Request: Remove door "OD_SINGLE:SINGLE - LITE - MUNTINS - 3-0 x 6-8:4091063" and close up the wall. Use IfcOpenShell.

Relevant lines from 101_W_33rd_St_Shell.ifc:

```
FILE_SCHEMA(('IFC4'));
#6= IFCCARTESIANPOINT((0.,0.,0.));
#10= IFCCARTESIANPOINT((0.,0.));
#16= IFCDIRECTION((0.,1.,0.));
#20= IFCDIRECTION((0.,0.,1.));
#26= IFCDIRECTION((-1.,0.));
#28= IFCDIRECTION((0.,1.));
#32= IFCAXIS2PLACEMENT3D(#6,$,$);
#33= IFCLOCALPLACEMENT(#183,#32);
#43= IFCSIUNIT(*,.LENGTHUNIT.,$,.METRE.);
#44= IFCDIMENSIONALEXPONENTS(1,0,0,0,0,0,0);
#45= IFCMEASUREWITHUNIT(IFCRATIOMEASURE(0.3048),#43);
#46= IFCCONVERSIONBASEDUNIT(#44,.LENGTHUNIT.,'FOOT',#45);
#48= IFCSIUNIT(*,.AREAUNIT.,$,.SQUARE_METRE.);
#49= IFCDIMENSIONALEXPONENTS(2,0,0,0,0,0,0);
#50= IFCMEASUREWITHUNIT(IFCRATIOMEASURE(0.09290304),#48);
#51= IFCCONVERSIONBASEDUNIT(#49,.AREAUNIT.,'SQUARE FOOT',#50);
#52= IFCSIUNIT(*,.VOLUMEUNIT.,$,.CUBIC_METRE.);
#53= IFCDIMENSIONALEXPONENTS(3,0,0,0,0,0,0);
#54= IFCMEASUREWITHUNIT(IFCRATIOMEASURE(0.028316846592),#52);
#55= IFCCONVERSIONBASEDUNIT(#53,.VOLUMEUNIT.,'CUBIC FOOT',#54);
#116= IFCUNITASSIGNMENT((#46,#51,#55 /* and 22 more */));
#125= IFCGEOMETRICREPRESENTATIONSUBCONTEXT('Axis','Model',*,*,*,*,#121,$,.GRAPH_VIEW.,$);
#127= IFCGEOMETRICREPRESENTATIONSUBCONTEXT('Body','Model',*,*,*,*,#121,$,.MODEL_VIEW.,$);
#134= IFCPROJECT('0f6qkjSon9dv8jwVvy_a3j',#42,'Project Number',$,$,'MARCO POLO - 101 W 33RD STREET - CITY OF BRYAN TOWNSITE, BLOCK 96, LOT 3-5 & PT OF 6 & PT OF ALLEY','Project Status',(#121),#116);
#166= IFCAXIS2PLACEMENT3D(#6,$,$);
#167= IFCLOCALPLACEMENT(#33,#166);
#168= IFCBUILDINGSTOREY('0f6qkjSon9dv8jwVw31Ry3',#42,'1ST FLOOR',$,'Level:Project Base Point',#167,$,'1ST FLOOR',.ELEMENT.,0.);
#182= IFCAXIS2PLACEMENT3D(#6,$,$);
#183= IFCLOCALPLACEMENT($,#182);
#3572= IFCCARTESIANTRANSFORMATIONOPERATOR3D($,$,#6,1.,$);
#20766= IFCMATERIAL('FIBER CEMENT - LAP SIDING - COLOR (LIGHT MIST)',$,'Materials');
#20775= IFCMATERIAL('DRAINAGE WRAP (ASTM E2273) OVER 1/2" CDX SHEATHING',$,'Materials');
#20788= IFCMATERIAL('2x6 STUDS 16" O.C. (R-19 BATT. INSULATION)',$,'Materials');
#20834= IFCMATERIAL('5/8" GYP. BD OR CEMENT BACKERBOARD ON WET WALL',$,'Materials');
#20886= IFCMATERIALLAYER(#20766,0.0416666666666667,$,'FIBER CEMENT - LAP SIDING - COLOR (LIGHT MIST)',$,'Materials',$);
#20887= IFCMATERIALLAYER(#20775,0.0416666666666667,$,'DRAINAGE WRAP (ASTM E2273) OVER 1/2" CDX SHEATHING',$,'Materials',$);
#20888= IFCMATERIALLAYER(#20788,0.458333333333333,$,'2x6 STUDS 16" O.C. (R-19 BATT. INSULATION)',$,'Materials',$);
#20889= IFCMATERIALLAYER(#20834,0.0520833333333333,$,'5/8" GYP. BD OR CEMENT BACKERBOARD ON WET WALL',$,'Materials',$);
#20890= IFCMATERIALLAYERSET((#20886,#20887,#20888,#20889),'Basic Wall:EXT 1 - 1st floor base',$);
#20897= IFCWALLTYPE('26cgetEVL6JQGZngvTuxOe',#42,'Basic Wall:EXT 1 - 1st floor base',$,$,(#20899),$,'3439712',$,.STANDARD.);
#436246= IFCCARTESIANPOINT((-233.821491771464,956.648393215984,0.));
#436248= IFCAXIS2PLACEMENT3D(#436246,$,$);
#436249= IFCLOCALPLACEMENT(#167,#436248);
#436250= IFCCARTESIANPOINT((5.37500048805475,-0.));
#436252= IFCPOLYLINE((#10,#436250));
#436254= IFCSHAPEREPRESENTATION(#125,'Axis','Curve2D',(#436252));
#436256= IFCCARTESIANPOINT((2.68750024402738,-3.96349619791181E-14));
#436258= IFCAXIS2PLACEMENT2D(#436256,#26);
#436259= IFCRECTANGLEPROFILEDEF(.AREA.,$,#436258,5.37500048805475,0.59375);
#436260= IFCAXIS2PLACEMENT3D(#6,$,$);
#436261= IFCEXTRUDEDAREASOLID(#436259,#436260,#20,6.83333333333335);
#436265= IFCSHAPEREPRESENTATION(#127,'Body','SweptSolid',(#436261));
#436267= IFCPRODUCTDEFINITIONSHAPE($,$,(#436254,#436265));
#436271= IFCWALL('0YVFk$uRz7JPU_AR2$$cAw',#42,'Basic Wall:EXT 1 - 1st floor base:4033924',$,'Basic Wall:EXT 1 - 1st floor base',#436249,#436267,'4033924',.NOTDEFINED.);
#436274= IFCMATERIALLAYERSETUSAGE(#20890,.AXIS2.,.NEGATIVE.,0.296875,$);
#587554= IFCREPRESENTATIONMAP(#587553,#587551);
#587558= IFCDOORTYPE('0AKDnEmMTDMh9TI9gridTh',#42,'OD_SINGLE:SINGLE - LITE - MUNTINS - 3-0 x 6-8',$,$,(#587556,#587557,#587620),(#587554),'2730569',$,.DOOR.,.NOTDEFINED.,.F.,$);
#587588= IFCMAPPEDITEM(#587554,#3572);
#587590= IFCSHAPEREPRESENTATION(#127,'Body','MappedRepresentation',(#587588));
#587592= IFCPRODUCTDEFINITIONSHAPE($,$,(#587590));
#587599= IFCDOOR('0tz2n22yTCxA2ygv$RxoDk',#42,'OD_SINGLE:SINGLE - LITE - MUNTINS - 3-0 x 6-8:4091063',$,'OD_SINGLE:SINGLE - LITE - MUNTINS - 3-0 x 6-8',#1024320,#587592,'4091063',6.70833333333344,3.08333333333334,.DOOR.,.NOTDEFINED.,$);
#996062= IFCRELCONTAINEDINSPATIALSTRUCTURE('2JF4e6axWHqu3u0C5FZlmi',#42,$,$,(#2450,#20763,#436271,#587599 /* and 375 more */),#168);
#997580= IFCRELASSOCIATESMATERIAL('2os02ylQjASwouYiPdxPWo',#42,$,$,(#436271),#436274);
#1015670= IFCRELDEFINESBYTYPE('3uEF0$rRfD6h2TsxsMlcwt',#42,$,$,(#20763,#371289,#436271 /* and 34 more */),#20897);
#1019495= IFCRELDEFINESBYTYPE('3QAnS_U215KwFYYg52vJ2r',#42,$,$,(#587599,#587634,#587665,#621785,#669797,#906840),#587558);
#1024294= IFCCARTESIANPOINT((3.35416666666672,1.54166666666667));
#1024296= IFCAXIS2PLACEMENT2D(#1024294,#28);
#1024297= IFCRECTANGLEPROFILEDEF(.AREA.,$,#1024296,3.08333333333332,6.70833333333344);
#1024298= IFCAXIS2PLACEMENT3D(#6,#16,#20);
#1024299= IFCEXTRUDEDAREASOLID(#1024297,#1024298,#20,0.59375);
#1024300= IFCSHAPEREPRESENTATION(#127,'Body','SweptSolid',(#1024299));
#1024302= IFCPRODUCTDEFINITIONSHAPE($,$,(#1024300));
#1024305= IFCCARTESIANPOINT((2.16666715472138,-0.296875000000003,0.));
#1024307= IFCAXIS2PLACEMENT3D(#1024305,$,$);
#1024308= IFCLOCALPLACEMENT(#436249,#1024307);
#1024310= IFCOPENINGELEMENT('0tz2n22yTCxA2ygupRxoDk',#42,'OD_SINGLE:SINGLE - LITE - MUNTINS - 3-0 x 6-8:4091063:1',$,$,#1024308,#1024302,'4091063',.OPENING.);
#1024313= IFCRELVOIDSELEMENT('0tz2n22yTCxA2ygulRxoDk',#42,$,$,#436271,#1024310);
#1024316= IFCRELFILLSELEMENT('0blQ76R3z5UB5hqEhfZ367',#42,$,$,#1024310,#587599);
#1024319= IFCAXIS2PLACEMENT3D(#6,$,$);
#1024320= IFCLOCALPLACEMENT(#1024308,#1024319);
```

```python
import ifcopenshell
import ifcopenshell.api.feature
import ifcopenshell.api.root
import ifcopenshell.geom
import ifcopenshell.util.shape

model = ifcopenshell.open("101_W_33rd_St_Shell.ifc")
settings = ifcopenshell.geom.settings()


def volume(element):
    """Net volume in cubic metres, openings subtracted."""
    shape = ifcopenshell.geom.create_shape(settings, element)
    return ifcopenshell.util.shape.get_volume(shape.geometry)


door = model.by_guid("0tz2n22yTCxA2ygv$RxoDk")
opening = door.FillsVoids[0].RelatingOpeningElement
wall = opening.VoidsElements[0].RelatingBuildingElement
before = volume(wall)

ifcopenshell.api.root.remove_product(model, product=door)
ifcopenshell.api.feature.remove_feature(model, feature=opening)

after = volume(wall)

print(f"wall volume {before:.3f} -> {after:.3f} m3")

model.write("101_W_33rd_St_Shell_edited.ifc")
```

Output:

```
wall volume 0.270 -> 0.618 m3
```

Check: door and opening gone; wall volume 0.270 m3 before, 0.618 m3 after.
